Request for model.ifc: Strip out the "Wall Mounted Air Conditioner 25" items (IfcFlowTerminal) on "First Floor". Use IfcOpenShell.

First a look at what the model holds.

```python
import ifcopenshell
import ifcopenshell.util.element

model = ifcopenshell.open("model.ifc")
print(model.schema)
storey = next(s for s in model.by_type("IfcBuildingStorey") if s.Name == "First Floor")
terminals = [e for e in ifcopenshell.util.element.get_decomposition(storey) if e.is_a("IfcFlowTerminal")]
seen = {}
for e in terminals:
    element_type = ifcopenshell.util.element.get_type(e)
    name = element_type.Name if element_type not in (None, e) else None
    seen[name] = seen.get(name, 0) + 1
for name, count in sorted(seen.items(), key=str):
    print(count, "x", name)
```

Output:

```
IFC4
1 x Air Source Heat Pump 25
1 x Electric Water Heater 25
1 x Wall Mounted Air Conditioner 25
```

```python
import ifcopenshell
import ifcopenshell.api.root
import ifcopenshell.util.element

model = ifcopenshell.open("model.ifc")

storey = next(s for s in model.by_type("IfcBuildingStorey") if s.Name == "First Floor")
terminals = [e for e in ifcopenshell.util.element.get_decomposition(storey) if e.is_a("IfcFlowTerminal")]
targets = [e for e in terminals if (t := ifcopenshell.util.element.get_type(e)) not in (None, e) and t.Name == "Wall Mounted Air Conditioner 25"]

for e in targets:
    ifcopenshell.api.root.remove_product(model, product=e)
print(len(targets), "removed")

model.write("model_rev.ifc")
```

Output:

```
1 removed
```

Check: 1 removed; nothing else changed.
